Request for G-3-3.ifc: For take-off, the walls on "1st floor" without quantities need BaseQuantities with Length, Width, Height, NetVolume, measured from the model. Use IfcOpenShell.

First a look at what the model holds.

```python
import ifcopenshell
import ifcopenshell.util.element
import ifcopenshell.util.unit

model = ifcopenshell.open("G-3-3.ifc")
print(model.schema)
for unit_type in ("LENGTHUNIT", "AREAUNIT", "VOLUMEUNIT"):
    print(unit_type, ifcopenshell.util.unit.calculate_unit_scale(model, unit_type))
storey = next(s for s in model.by_type("IfcBuildingStorey") if s.Name == "1st floor")
walls = [e for e in ifcopenshell.util.element.get_decomposition(storey) if e.is_a("IfcWall")]
for e in sorted(walls, key=lambda e: e.id()):
    print(e.id(), e.is_a(), e.Name, list(ifcopenshell.util.element.get_psets(e, qtos_only=True)), sep=" | ")
```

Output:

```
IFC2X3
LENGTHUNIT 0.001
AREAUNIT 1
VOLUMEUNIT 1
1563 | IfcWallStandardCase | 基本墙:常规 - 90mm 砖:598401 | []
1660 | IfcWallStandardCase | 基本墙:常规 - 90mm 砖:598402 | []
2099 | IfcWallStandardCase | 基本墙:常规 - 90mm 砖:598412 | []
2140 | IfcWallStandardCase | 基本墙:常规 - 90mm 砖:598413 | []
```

```python
import ifcopenshell
import ifcopenshell.api.pset
import ifcopenshell.geom
import ifcopenshell.util.element
import ifcopenshell.util.shape
import ifcopenshell.util.unit

model = ifcopenshell.open("G-3-3.ifc")
unit_scale = ifcopenshell.util.unit.calculate_unit_scale(model)
volume_scale = ifcopenshell.util.unit.calculate_unit_scale(model, "VOLUMEUNIT")
settings = ifcopenshell.geom.settings()

storey = next(s for s in model.by_type("IfcBuildingStorey") if s.Name == "1st floor")
walls = [e for e in ifcopenshell.util.element.get_decomposition(storey) if e.is_a("IfcWall")]

for e in sorted(walls, key=lambda e: e.id()):
    if ifcopenshell.util.element.get_psets(e, qtos_only=True, should_inherit=False):
        continue
    # Geometry comes back in metres, in the element's own axes.
    shape = ifcopenshell.geom.create_shape(settings, e)
    values = {
        "Length": ifcopenshell.util.shape.get_x(shape.geometry) / unit_scale,
        "Width": ifcopenshell.util.shape.get_y(shape.geometry) / unit_scale,
        "Height": ifcopenshell.util.shape.get_z(shape.geometry) / unit_scale,
        "NetVolume": ifcopenshell.util.shape.get_volume(shape.geometry) / volume_scale,
    }
    qto = ifcopenshell.api.pset.add_qto(model, product=e, name="BaseQuantities")
    ifcopenshell.api.pset.edit_qto(model, qto=qto, properties=values)
    print(e.id(), {k: round(v, 3) for k, v in values.items()})

model.write("G-3-3-out.ifc")
```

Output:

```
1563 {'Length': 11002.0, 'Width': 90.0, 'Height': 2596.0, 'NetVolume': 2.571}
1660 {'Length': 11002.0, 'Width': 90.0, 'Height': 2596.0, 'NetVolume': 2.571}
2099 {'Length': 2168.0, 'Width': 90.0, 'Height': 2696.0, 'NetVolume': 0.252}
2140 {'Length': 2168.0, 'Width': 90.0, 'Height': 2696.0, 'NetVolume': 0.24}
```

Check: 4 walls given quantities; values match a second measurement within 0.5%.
